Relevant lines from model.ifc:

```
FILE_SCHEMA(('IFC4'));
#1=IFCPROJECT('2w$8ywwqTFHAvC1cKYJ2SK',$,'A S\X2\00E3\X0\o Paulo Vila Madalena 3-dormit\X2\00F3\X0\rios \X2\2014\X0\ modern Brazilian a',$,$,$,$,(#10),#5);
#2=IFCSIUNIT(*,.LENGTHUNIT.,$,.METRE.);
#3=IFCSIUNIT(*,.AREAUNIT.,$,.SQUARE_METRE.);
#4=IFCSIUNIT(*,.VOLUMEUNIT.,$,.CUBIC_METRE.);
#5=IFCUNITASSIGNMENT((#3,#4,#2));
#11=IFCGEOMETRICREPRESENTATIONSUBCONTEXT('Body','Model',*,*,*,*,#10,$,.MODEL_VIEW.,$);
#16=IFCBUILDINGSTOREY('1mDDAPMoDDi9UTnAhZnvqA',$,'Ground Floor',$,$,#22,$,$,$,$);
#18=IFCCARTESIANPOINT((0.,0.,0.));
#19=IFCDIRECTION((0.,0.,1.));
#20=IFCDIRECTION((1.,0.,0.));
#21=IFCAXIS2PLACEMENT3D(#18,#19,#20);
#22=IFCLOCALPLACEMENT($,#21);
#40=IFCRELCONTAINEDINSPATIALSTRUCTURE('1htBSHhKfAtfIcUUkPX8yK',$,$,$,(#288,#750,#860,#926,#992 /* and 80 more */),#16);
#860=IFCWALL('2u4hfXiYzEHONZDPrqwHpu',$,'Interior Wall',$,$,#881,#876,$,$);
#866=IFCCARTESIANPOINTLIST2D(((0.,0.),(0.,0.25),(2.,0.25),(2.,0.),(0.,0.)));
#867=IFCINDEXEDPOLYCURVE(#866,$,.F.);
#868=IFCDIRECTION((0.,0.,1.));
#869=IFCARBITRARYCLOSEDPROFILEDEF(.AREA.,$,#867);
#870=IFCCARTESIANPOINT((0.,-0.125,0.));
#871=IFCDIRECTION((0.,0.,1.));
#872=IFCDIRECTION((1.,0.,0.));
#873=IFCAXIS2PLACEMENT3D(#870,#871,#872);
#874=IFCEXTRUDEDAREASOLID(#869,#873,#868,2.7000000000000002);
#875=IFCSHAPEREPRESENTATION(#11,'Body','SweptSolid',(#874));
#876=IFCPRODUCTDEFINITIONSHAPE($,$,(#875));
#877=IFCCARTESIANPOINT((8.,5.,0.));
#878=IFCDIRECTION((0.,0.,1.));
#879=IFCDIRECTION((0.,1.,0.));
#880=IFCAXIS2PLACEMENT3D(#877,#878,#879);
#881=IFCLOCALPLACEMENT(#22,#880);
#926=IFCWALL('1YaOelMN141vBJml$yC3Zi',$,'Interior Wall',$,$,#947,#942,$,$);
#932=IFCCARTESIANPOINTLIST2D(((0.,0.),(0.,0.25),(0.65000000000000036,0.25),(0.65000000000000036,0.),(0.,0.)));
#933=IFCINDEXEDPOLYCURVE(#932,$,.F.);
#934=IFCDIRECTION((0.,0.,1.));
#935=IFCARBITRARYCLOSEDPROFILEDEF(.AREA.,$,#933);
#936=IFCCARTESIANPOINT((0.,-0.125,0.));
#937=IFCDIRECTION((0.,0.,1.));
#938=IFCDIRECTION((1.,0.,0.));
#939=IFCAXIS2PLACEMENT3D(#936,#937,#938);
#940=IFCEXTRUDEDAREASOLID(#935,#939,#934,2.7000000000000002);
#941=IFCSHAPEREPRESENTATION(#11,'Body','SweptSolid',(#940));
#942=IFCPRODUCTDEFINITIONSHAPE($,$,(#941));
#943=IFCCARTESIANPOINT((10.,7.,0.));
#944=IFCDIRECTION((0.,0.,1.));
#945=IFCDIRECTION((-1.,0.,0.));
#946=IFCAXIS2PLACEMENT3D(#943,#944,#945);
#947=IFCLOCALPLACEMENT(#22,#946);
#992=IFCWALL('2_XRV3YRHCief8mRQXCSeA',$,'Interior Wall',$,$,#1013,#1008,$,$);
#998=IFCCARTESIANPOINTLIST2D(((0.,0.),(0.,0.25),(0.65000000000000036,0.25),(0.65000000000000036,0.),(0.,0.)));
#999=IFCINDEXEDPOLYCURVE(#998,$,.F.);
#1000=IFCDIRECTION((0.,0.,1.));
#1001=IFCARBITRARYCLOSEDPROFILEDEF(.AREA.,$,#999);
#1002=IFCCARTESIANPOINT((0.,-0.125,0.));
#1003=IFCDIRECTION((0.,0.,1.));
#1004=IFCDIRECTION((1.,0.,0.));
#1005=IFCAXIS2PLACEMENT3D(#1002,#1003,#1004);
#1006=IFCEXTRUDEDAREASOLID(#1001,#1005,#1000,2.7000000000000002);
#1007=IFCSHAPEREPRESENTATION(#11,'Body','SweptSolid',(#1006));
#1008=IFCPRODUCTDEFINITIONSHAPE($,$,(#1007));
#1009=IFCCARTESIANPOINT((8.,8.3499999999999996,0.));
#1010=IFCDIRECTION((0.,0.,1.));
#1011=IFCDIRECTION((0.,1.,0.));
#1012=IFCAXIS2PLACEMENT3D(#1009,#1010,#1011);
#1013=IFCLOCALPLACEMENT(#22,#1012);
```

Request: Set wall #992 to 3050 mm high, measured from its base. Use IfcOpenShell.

```python
import ifcopenshell
import ifcopenshell.geom
import ifcopenshell.util.representation
import ifcopenshell.util.shape
import ifcopenshell.util.unit

model = ifcopenshell.open("model.ifc")
unit_scale = ifcopenshell.util.unit.calculate_unit_scale(model)
settings = ifcopenshell.geom.settings()


def volume(element):
    """Net volume in cubic metres, openings subtracted."""
    shape = ifcopenshell.geom.create_shape(settings, element)
    return ifcopenshell.util.shape.get_volume(shape.geometry)


wall = model.by_guid("2_XRV3YRHCief8mRQXCSeA")
before = volume(wall)

body = ifcopenshell.util.representation.get_representation(wall, "Model", "Body")
solid = body.Items[0]
old_height = solid.Depth
solid.Depth = 3.05 / unit_scale
after = volume(wall)

print(f"height {old_height:g} -> {solid.Depth:g}, volume {before:.3f} -> {after:.3f} m3")

model.write("model_edited.ifc")
```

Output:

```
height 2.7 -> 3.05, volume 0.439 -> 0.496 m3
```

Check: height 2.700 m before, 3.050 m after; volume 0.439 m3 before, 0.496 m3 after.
